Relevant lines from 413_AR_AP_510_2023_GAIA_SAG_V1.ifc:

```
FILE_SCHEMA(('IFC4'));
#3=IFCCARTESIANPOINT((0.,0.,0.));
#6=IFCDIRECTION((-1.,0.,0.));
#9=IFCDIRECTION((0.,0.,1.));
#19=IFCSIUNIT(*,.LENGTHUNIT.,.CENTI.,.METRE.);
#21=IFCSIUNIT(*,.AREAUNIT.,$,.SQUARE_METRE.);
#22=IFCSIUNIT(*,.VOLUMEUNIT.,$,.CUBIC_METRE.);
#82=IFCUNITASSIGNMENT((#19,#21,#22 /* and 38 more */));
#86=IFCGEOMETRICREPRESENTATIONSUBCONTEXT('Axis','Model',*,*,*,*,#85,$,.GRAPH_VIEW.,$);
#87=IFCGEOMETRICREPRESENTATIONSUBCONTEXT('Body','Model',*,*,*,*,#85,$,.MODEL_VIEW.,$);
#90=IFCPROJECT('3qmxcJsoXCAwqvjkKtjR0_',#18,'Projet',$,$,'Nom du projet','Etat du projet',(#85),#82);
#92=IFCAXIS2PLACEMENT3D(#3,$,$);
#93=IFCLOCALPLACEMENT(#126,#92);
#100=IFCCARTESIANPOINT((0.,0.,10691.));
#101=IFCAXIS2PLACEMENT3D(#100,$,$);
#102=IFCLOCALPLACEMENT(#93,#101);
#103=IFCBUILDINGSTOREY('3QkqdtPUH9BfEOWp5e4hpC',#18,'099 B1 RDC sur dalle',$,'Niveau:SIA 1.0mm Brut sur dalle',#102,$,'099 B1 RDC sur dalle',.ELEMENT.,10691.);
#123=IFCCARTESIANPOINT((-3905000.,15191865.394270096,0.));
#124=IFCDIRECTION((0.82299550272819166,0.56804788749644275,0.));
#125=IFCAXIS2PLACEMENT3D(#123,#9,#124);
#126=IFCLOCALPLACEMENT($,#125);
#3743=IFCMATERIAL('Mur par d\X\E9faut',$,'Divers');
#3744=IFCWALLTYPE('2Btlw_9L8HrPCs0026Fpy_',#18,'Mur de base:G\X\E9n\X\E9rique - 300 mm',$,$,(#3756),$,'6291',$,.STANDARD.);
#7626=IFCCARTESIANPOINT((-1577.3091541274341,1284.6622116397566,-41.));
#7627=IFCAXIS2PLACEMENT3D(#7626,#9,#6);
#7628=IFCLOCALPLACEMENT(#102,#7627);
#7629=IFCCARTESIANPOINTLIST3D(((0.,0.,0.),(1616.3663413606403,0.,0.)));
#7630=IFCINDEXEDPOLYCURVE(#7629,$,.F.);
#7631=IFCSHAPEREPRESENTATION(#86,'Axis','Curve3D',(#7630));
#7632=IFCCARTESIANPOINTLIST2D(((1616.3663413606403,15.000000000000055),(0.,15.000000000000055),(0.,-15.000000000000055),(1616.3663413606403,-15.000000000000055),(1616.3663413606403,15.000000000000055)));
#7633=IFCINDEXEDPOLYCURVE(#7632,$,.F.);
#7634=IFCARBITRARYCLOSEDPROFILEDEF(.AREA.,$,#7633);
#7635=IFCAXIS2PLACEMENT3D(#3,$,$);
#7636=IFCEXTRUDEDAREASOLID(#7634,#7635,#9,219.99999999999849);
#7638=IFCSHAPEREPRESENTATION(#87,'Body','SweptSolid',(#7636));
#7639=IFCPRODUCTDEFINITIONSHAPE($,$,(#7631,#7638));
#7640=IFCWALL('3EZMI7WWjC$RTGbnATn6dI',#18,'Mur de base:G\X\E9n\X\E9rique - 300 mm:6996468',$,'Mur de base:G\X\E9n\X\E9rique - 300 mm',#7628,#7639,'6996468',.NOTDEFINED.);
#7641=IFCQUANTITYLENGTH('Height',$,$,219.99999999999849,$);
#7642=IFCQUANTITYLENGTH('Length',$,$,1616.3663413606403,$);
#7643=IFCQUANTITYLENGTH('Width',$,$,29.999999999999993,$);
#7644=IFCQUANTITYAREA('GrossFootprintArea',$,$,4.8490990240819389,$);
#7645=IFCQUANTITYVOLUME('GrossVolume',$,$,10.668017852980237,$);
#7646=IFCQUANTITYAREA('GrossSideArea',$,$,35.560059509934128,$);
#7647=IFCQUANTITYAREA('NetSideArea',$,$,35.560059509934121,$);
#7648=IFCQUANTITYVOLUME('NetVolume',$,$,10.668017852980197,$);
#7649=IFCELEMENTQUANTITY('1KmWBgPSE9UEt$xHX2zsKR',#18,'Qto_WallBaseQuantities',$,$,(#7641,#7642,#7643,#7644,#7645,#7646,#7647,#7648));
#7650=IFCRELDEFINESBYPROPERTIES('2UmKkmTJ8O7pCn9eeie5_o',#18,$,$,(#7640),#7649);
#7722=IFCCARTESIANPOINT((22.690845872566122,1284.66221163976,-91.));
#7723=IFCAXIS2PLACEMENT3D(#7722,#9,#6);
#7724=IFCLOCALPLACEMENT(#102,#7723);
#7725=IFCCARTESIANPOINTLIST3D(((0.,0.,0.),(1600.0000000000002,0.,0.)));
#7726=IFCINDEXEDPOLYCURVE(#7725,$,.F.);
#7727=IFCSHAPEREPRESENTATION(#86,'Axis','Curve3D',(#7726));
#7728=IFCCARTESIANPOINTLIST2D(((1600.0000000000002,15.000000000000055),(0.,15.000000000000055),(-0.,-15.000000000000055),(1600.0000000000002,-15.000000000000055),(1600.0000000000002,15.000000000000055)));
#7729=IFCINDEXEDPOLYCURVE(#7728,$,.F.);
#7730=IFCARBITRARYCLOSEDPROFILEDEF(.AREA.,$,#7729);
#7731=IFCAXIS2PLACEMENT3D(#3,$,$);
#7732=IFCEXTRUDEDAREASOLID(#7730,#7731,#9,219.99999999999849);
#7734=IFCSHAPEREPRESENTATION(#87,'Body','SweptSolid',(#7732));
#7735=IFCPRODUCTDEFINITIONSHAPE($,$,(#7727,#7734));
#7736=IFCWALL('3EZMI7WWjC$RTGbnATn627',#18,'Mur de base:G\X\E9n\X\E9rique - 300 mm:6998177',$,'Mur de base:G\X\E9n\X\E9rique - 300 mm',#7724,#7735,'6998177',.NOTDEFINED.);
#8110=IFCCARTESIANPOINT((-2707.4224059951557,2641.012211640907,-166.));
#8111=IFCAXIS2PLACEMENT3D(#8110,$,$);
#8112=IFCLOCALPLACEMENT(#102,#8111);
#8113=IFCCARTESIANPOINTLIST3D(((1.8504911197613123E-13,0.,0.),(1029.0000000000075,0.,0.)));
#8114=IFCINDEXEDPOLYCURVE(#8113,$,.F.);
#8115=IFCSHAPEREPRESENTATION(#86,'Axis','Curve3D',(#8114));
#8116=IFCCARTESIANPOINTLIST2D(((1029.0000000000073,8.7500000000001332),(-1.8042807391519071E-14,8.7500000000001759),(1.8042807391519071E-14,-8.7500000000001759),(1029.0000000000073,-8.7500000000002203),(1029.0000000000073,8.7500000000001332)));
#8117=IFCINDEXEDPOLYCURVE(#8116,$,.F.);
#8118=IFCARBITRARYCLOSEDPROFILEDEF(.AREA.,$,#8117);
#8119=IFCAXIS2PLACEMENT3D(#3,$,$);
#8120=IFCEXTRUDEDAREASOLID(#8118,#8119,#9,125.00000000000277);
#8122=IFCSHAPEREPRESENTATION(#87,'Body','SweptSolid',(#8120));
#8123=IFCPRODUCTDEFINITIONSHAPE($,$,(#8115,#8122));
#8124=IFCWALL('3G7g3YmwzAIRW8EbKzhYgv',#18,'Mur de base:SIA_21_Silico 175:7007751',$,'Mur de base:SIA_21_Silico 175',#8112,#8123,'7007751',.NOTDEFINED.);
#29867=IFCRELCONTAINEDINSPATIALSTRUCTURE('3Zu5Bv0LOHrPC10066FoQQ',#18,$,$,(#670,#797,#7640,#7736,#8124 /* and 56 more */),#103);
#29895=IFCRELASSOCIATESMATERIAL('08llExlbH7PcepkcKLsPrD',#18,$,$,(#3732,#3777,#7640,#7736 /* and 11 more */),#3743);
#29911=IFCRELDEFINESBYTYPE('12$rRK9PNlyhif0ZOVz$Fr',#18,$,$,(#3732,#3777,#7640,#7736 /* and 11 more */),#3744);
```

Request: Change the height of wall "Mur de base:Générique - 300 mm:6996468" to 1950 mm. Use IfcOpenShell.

```python
import ifcopenshell
import ifcopenshell.api.pset
import ifcopenshell.geom
import ifcopenshell.util.element
import ifcopenshell.util.representation
import ifcopenshell.util.shape
import ifcopenshell.util.unit

model = ifcopenshell.open("413_AR_AP_510_2023_GAIA_SAG_V1.ifc")
unit_scale = ifcopenshell.util.unit.calculate_unit_scale(model)
area_scale = ifcopenshell.util.unit.calculate_unit_scale(model, "AREAUNIT")
volume_scale = ifcopenshell.util.unit.calculate_unit_scale(model, "VOLUMEUNIT")
settings = ifcopenshell.geom.settings()


def volume(element):
    """Net volume in cubic metres, openings subtracted."""
    shape = ifcopenshell.geom.create_shape(settings, element)
    return ifcopenshell.util.shape.get_volume(shape.geometry)


wall = model.by_guid("3EZMI7WWjC$RTGbnATn6dI")
before = volume(wall)

body = ifcopenshell.util.representation.get_representation(wall, "Model", "Body")
solid = body.Items[0]
old_height = solid.Depth
solid.Depth = 1.95 / unit_scale
after = volume(wall)
thickness = 0.3  # wall thickness in metres

# Update the stored height, areas and volumes.
qto = model.by_id(ifcopenshell.util.element.get_pset(wall, "Qto_WallBaseQuantities", should_inherit=False)["id"])
ifcopenshell.api.pset.edit_qto(model, qto=qto, properties={
    "Height": solid.Depth,
    "GrossVolume": ifcopenshell.util.element.get_pset(wall, "Qto_WallBaseQuantities", "GrossVolume") * solid.Depth / old_height,
    "GrossSideArea": ifcopenshell.util.element.get_pset(wall, "Qto_WallBaseQuantities", "GrossSideArea") * solid.Depth / old_height,
    "NetSideArea": after / thickness / area_scale,
    "NetVolume": after / volume_scale,
})

print(f"height {old_height:g} -> {solid.Depth:g}, volume {before:.3f} -> {after:.3f} m3")

model.write("413_AR_AP_510_2023_GAIA_SAG_V1-out.ifc")
```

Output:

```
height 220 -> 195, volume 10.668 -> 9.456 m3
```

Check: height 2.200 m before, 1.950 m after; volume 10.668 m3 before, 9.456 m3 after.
